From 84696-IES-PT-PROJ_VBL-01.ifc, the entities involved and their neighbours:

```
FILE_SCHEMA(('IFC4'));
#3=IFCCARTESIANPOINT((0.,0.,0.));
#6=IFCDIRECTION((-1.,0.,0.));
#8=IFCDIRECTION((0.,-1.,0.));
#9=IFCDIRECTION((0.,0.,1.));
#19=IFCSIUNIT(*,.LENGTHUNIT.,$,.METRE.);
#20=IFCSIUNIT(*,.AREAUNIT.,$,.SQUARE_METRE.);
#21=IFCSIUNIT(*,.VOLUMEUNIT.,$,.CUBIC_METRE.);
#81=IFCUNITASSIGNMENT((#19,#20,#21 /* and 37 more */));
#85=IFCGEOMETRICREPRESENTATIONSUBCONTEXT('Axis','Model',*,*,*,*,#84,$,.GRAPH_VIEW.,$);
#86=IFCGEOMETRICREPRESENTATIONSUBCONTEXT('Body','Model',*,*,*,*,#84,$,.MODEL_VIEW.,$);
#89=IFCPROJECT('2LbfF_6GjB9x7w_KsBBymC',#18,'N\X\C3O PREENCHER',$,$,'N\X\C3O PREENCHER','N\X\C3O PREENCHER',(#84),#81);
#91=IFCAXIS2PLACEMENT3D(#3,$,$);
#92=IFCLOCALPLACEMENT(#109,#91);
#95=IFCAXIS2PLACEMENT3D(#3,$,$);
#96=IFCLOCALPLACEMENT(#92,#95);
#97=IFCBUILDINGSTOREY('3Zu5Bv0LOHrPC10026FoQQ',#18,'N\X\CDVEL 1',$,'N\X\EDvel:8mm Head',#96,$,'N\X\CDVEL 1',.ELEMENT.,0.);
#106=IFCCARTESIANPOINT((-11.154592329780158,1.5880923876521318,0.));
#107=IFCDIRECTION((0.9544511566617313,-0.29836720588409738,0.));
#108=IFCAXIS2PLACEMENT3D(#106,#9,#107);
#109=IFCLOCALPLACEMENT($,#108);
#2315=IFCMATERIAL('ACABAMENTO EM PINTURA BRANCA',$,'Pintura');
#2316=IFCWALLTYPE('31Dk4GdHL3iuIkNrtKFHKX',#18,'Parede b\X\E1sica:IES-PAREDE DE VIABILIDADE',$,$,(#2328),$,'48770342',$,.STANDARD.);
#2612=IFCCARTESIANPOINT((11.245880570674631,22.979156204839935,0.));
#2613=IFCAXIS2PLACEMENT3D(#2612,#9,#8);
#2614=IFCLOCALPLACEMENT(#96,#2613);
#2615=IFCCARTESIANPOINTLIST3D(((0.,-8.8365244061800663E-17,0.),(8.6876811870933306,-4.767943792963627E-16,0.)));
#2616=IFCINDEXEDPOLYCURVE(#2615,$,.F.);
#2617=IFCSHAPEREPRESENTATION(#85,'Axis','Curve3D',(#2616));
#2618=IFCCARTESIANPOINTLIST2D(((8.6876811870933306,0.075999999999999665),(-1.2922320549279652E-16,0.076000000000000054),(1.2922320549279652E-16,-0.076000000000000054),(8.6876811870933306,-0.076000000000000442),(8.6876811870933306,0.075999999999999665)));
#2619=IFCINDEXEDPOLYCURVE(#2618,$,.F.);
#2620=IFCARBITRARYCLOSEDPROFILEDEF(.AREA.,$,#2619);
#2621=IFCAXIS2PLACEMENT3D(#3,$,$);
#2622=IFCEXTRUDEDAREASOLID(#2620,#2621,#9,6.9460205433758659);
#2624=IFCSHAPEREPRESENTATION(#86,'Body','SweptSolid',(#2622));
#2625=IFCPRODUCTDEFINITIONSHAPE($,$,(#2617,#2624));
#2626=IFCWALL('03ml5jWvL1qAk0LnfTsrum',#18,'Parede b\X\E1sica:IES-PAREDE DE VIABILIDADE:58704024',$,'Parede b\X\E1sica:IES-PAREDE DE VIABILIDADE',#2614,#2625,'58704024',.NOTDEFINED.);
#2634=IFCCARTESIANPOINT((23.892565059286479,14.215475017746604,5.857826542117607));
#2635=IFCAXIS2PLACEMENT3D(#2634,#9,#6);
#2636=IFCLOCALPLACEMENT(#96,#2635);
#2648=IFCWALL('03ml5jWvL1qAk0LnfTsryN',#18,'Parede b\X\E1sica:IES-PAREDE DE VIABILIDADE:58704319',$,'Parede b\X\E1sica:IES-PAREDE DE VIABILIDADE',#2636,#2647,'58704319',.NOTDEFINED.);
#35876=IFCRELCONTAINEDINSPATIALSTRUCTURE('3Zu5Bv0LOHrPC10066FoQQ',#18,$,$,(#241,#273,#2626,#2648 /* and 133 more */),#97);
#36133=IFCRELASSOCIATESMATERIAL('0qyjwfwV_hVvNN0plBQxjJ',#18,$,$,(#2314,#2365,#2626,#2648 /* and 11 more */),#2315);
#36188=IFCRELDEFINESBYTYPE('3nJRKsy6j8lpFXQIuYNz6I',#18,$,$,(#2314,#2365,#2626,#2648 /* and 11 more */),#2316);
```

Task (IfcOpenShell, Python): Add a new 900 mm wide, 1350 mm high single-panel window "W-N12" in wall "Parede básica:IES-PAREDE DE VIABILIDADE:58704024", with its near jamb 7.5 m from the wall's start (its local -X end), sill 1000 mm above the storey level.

```python
import numpy as np
import ifcopenshell
import ifcopenshell.api.feature
import ifcopenshell.api.geometry
import ifcopenshell.api.root
import ifcopenshell.api.spatial
import ifcopenshell.geom
import ifcopenshell.util.element
import ifcopenshell.util.placement
import ifcopenshell.util.representation
import ifcopenshell.util.shape
import ifcopenshell.util.unit

model = ifcopenshell.open("84696-IES-PT-PROJ_VBL-01.ifc")
unit_scale = ifcopenshell.util.unit.calculate_unit_scale(model)
settings = ifcopenshell.geom.settings()


def volume(element):
    """Net volume in cubic metres, openings subtracted."""
    shape = ifcopenshell.geom.create_shape(settings, element)
    return ifcopenshell.util.shape.get_volume(shape.geometry)


wall = model.by_guid("03ml5jWvL1qAk0LnfTsrum")
storey = ifcopenshell.util.element.get_container(wall, ifc_class="IfcBuildingStorey")
context = ifcopenshell.util.representation.get_context(model, "Model", "Body", "MODEL_VIEW")
before = volume(wall)

width, height, from_end, sill = 0.9, 1.35, 7.5, 1  # metres

# The wall runs along its own X axis, and the end named is its -X end.
wall_shape = ifcopenshell.geom.create_shape(settings, wall)
x, y, z = ifcopenshell.util.shape.get_vertices(wall_shape.geometry).T
start = x.min() + from_end
face, thickness = float(y.min()), float(y.max() - y.min())
wall_matrix = ifcopenshell.util.placement.get_local_placement(wall.ObjectPlacement)
level = ifcopenshell.util.placement.get_local_placement(storey.ObjectPlacement)[2, 3]


def in_wall(x, y):
    """Placement at x, y metres in the wall's axes, at sill height."""
    matrix = wall_matrix.copy()
    matrix[:, 3] = wall_matrix @ np.array([x / unit_scale, y / unit_scale, 0.0, 1.0])
    matrix[2, 3] = level + sill / unit_scale
    return matrix


# Opening: a box that overshoots both wall faces by 50 mm.
opening = ifcopenshell.api.root.create_entity(model, ifc_class="IfcOpeningElement", predefined_type="OPENING")
box = ifcopenshell.api.geometry.add_wall_representation(
    model, context=context, length=width, height=height, thickness=thickness + 0.1
)
ifcopenshell.api.geometry.assign_representation(model, product=opening, representation=box)
ifcopenshell.api.geometry.edit_object_placement(model, product=opening, matrix=in_wall(start, face - 0.05), is_si=False)
ifcopenshell.api.feature.add_feature(model, feature=opening, element=wall)

window = ifcopenshell.api.root.create_entity(model, ifc_class="IfcWindow", name="W-N12", predefined_type="WINDOW")
window.OverallWidth, window.OverallHeight = width / unit_scale, height / unit_scale
window.PartitioningType = "SINGLE_PANEL"
body = ifcopenshell.api.geometry.add_window_representation(
    model,
    context=context,
    overall_width=window.OverallWidth,
    overall_height=window.OverallHeight,
    partition_type="SINGLE_PANEL",
)
ifcopenshell.api.geometry.assign_representation(model, product=window, representation=body)
ifcopenshell.api.spatial.assign_container(model, products=[window], relating_structure=storey)
ifcopenshell.api.feature.add_filling(model, opening=opening, element=window)

# Centre the window in the wall's thickness.
ifcopenshell.api.geometry.edit_object_placement(model, product=window, matrix=in_wall(start, face), is_si=False)
window_shape = ifcopenshell.geom.create_shape(settings, window)
depth = ifcopenshell.util.shape.get_vertices(window_shape.geometry)[:, 1]
offset = face + thickness / 2 - (depth.min() + depth.max()) / 2
ifcopenshell.api.geometry.edit_object_placement(model, product=window, matrix=in_wall(start, offset), is_si=False)

after = volume(wall)

print(f"wall volume {before:.3f} -> {after:.3f} m3")

model.write("84696-IES-PT-PROJ_VBL-01-out.ifc")
```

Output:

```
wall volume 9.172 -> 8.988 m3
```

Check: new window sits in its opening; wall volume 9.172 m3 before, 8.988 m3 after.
